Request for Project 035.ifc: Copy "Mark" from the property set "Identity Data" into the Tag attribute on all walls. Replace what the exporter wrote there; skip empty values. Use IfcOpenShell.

First a look at what the model holds.

```python
import ifcopenshell
import ifcopenshell.util.element

model = ifcopenshell.open("Project 035.ifc")
print(model.schema)
walls = model.by_type("IfcWall")
print(len(walls), "walls")
for e in walls[:8]:
    source = ifcopenshell.util.element.get_pset(e, "Identity Data", "Mark")
    target = e.Tag
    print(e.id(), repr(source), repr(target), sep=" | ")
```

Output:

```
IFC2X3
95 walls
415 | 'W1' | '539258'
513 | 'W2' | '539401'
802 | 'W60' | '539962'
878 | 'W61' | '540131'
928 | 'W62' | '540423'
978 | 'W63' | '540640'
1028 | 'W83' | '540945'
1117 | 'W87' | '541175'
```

```python
import ifcopenshell
import ifcopenshell.util.element

model = ifcopenshell.open("Project 035.ifc")

count = 0
for e in model.by_type("IfcWall"):
    value = ifcopenshell.util.element.get_pset(e, "Identity Data", "Mark")
    current = e.Tag
    if not value or not value.strip() or current == value:
        continue
    e.Tag = value
    count += 1

print(count, "walls updated")

model.write("Project 035_rev.ifc")
```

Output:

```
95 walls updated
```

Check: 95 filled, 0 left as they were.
